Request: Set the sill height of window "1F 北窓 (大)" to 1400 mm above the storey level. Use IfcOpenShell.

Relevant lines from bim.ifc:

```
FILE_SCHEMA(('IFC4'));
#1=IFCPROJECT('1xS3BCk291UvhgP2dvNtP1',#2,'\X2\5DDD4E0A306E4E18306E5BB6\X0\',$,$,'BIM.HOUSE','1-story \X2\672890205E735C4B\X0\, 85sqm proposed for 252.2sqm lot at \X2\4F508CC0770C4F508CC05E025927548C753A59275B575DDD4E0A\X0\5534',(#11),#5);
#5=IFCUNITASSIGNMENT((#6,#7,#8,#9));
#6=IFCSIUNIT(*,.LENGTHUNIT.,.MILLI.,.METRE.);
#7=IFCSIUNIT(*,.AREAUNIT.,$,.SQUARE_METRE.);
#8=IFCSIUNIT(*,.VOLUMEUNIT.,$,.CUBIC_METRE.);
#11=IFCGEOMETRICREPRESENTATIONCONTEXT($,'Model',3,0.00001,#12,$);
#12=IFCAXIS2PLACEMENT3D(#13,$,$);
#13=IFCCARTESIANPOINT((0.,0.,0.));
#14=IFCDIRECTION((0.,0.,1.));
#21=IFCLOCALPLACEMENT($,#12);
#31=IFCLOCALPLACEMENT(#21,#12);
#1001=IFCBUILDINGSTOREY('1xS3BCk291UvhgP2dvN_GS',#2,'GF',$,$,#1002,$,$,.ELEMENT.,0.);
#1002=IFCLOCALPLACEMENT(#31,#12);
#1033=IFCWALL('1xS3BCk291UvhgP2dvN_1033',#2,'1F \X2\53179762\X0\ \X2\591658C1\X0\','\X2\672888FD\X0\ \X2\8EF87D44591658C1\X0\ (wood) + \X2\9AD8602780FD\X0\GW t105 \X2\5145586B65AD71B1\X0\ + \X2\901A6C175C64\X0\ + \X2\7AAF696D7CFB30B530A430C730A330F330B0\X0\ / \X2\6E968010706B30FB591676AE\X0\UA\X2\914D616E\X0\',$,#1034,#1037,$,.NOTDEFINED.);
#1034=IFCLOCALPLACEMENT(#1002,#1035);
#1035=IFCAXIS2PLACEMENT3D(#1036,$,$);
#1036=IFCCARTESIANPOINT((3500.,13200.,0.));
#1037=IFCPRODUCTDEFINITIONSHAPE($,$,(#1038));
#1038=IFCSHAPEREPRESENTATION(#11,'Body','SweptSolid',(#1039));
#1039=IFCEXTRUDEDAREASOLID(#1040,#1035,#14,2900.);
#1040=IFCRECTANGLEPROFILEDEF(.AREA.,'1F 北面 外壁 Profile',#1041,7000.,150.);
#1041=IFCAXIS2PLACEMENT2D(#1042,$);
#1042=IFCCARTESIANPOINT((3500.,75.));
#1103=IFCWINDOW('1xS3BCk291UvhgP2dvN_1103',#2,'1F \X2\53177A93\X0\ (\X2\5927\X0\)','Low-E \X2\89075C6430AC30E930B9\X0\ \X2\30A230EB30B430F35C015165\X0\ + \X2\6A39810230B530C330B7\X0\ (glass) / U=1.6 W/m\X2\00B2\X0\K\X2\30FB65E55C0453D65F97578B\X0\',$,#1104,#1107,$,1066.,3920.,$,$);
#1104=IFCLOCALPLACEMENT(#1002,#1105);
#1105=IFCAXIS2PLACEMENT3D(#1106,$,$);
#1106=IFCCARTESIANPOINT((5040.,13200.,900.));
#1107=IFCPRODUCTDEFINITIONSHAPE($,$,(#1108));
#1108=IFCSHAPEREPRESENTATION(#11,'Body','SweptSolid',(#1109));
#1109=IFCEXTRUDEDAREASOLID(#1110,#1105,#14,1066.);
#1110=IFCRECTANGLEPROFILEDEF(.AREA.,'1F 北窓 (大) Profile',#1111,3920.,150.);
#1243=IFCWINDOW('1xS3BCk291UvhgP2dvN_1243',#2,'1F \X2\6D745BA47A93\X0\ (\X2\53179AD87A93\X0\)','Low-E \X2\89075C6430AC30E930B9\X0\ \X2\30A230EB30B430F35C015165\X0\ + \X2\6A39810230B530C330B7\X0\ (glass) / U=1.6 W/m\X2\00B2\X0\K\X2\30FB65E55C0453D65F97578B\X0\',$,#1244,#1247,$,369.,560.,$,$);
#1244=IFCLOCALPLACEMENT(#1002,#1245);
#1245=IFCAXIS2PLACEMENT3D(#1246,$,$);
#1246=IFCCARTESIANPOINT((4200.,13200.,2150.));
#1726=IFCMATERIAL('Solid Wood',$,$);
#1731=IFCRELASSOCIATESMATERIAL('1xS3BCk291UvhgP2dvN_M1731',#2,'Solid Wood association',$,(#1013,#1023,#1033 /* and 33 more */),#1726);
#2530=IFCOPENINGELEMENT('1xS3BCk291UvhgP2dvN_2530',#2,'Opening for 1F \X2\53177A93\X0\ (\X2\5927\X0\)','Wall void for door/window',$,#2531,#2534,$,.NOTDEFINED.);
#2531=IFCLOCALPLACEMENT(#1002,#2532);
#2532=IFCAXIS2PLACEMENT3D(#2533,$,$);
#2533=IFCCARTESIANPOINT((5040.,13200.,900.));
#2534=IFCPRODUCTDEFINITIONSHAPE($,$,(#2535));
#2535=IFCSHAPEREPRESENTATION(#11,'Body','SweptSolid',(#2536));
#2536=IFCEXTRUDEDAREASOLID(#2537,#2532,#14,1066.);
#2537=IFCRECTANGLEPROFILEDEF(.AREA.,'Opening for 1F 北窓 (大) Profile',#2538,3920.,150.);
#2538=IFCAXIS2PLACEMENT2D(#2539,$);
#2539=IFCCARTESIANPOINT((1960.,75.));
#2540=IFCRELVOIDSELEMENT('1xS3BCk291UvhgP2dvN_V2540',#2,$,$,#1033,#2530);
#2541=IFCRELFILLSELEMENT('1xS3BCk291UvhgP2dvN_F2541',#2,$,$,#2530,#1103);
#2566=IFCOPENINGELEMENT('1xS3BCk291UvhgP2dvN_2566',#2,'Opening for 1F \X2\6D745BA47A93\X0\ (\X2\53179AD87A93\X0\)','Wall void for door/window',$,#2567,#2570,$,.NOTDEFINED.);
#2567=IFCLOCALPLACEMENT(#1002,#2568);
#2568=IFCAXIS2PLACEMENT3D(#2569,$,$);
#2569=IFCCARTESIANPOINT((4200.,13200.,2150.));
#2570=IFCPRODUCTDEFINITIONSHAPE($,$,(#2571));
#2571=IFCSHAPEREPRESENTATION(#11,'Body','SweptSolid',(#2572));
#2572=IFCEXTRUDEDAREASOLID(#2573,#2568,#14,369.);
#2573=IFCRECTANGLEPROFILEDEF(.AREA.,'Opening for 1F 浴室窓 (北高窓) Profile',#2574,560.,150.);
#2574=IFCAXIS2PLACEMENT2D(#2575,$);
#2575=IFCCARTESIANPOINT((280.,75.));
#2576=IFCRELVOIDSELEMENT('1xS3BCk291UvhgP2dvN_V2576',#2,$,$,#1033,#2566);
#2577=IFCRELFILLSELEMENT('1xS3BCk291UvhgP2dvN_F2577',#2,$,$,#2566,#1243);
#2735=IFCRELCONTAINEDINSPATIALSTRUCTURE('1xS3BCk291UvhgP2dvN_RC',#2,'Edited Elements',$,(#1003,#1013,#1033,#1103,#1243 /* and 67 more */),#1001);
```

```python
import numpy as np
import ifcopenshell
import ifcopenshell.api.geometry
import ifcopenshell.geom
import ifcopenshell.util.element
import ifcopenshell.util.placement
import ifcopenshell.util.shape
import ifcopenshell.util.unit

model = ifcopenshell.open("bim.ifc")
unit_scale = ifcopenshell.util.unit.calculate_unit_scale(model)

window = model.by_guid("1xS3BCk291UvhgP2dvN_1103")
opening = window.FillsVoids[0].RelatingOpeningElement
storey = ifcopenshell.util.element.get_container(window, ifc_class="IfcBuildingStorey")
level = ifcopenshell.util.placement.get_local_placement(storey.ObjectPlacement)[2, 3]

# The opening's origin need not be at the sill, so measure its lowest point.
shape = ifcopenshell.geom.create_shape(ifcopenshell.geom.settings(), opening)
bottom = ifcopenshell.util.shape.get_shape_bottom_elevation(shape, shape.geometry) / unit_scale
dz = level + 1.4 / unit_scale - bottom

shift = np.array([0.0, 0.0, dz])
# The window is not placed relative to its opening, so move both.
for product in (opening, window):
    matrix = ifcopenshell.util.placement.get_local_placement(product.ObjectPlacement)
    matrix[:3, 3] += shift
    ifcopenshell.api.geometry.edit_object_placement(model, product=product, matrix=matrix, is_si=False)

print(f"moved by {dz * unit_scale:+.3f} m")

model.write("bim_edited.ifc")
```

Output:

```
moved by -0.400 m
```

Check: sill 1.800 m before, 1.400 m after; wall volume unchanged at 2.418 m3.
